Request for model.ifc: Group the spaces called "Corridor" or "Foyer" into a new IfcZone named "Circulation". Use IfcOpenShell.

First a look at what the model holds.

```python
import ifcopenshell

model = ifcopenshell.open("model.ifc")
print(model.schema)
seen = {}
for space in model.by_type("IfcSpace"):
    seen[space.LongName] = seen.get(space.LongName, 0) + 1
for name, count in sorted(seen.items(), key=str):
    print(count, "x", name)
print("zones:", [z.Name for z in model.by_type("IfcZone")][:20])
```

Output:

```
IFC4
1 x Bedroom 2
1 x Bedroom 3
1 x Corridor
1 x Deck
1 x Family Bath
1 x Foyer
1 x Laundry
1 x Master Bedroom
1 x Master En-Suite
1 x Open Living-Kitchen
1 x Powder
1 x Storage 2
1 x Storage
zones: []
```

```python
import ifcopenshell
import ifcopenshell.api.group
import ifcopenshell.api.root

model = ifcopenshell.open("model.ifc")

names = {"Corridor", "Foyer"}
spaces = [s for s in model.by_type("IfcSpace") if s.LongName in names]

zone = ifcopenshell.api.root.create_entity(model, ifc_class="IfcZone", name="Circulation")
ifcopenshell.api.group.assign_group(model, products=spaces, group=zone)
print(len(spaces), "spaces in", zone.Name)

model.write("model_edited.ifc")
```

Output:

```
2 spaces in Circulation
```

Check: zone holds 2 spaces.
